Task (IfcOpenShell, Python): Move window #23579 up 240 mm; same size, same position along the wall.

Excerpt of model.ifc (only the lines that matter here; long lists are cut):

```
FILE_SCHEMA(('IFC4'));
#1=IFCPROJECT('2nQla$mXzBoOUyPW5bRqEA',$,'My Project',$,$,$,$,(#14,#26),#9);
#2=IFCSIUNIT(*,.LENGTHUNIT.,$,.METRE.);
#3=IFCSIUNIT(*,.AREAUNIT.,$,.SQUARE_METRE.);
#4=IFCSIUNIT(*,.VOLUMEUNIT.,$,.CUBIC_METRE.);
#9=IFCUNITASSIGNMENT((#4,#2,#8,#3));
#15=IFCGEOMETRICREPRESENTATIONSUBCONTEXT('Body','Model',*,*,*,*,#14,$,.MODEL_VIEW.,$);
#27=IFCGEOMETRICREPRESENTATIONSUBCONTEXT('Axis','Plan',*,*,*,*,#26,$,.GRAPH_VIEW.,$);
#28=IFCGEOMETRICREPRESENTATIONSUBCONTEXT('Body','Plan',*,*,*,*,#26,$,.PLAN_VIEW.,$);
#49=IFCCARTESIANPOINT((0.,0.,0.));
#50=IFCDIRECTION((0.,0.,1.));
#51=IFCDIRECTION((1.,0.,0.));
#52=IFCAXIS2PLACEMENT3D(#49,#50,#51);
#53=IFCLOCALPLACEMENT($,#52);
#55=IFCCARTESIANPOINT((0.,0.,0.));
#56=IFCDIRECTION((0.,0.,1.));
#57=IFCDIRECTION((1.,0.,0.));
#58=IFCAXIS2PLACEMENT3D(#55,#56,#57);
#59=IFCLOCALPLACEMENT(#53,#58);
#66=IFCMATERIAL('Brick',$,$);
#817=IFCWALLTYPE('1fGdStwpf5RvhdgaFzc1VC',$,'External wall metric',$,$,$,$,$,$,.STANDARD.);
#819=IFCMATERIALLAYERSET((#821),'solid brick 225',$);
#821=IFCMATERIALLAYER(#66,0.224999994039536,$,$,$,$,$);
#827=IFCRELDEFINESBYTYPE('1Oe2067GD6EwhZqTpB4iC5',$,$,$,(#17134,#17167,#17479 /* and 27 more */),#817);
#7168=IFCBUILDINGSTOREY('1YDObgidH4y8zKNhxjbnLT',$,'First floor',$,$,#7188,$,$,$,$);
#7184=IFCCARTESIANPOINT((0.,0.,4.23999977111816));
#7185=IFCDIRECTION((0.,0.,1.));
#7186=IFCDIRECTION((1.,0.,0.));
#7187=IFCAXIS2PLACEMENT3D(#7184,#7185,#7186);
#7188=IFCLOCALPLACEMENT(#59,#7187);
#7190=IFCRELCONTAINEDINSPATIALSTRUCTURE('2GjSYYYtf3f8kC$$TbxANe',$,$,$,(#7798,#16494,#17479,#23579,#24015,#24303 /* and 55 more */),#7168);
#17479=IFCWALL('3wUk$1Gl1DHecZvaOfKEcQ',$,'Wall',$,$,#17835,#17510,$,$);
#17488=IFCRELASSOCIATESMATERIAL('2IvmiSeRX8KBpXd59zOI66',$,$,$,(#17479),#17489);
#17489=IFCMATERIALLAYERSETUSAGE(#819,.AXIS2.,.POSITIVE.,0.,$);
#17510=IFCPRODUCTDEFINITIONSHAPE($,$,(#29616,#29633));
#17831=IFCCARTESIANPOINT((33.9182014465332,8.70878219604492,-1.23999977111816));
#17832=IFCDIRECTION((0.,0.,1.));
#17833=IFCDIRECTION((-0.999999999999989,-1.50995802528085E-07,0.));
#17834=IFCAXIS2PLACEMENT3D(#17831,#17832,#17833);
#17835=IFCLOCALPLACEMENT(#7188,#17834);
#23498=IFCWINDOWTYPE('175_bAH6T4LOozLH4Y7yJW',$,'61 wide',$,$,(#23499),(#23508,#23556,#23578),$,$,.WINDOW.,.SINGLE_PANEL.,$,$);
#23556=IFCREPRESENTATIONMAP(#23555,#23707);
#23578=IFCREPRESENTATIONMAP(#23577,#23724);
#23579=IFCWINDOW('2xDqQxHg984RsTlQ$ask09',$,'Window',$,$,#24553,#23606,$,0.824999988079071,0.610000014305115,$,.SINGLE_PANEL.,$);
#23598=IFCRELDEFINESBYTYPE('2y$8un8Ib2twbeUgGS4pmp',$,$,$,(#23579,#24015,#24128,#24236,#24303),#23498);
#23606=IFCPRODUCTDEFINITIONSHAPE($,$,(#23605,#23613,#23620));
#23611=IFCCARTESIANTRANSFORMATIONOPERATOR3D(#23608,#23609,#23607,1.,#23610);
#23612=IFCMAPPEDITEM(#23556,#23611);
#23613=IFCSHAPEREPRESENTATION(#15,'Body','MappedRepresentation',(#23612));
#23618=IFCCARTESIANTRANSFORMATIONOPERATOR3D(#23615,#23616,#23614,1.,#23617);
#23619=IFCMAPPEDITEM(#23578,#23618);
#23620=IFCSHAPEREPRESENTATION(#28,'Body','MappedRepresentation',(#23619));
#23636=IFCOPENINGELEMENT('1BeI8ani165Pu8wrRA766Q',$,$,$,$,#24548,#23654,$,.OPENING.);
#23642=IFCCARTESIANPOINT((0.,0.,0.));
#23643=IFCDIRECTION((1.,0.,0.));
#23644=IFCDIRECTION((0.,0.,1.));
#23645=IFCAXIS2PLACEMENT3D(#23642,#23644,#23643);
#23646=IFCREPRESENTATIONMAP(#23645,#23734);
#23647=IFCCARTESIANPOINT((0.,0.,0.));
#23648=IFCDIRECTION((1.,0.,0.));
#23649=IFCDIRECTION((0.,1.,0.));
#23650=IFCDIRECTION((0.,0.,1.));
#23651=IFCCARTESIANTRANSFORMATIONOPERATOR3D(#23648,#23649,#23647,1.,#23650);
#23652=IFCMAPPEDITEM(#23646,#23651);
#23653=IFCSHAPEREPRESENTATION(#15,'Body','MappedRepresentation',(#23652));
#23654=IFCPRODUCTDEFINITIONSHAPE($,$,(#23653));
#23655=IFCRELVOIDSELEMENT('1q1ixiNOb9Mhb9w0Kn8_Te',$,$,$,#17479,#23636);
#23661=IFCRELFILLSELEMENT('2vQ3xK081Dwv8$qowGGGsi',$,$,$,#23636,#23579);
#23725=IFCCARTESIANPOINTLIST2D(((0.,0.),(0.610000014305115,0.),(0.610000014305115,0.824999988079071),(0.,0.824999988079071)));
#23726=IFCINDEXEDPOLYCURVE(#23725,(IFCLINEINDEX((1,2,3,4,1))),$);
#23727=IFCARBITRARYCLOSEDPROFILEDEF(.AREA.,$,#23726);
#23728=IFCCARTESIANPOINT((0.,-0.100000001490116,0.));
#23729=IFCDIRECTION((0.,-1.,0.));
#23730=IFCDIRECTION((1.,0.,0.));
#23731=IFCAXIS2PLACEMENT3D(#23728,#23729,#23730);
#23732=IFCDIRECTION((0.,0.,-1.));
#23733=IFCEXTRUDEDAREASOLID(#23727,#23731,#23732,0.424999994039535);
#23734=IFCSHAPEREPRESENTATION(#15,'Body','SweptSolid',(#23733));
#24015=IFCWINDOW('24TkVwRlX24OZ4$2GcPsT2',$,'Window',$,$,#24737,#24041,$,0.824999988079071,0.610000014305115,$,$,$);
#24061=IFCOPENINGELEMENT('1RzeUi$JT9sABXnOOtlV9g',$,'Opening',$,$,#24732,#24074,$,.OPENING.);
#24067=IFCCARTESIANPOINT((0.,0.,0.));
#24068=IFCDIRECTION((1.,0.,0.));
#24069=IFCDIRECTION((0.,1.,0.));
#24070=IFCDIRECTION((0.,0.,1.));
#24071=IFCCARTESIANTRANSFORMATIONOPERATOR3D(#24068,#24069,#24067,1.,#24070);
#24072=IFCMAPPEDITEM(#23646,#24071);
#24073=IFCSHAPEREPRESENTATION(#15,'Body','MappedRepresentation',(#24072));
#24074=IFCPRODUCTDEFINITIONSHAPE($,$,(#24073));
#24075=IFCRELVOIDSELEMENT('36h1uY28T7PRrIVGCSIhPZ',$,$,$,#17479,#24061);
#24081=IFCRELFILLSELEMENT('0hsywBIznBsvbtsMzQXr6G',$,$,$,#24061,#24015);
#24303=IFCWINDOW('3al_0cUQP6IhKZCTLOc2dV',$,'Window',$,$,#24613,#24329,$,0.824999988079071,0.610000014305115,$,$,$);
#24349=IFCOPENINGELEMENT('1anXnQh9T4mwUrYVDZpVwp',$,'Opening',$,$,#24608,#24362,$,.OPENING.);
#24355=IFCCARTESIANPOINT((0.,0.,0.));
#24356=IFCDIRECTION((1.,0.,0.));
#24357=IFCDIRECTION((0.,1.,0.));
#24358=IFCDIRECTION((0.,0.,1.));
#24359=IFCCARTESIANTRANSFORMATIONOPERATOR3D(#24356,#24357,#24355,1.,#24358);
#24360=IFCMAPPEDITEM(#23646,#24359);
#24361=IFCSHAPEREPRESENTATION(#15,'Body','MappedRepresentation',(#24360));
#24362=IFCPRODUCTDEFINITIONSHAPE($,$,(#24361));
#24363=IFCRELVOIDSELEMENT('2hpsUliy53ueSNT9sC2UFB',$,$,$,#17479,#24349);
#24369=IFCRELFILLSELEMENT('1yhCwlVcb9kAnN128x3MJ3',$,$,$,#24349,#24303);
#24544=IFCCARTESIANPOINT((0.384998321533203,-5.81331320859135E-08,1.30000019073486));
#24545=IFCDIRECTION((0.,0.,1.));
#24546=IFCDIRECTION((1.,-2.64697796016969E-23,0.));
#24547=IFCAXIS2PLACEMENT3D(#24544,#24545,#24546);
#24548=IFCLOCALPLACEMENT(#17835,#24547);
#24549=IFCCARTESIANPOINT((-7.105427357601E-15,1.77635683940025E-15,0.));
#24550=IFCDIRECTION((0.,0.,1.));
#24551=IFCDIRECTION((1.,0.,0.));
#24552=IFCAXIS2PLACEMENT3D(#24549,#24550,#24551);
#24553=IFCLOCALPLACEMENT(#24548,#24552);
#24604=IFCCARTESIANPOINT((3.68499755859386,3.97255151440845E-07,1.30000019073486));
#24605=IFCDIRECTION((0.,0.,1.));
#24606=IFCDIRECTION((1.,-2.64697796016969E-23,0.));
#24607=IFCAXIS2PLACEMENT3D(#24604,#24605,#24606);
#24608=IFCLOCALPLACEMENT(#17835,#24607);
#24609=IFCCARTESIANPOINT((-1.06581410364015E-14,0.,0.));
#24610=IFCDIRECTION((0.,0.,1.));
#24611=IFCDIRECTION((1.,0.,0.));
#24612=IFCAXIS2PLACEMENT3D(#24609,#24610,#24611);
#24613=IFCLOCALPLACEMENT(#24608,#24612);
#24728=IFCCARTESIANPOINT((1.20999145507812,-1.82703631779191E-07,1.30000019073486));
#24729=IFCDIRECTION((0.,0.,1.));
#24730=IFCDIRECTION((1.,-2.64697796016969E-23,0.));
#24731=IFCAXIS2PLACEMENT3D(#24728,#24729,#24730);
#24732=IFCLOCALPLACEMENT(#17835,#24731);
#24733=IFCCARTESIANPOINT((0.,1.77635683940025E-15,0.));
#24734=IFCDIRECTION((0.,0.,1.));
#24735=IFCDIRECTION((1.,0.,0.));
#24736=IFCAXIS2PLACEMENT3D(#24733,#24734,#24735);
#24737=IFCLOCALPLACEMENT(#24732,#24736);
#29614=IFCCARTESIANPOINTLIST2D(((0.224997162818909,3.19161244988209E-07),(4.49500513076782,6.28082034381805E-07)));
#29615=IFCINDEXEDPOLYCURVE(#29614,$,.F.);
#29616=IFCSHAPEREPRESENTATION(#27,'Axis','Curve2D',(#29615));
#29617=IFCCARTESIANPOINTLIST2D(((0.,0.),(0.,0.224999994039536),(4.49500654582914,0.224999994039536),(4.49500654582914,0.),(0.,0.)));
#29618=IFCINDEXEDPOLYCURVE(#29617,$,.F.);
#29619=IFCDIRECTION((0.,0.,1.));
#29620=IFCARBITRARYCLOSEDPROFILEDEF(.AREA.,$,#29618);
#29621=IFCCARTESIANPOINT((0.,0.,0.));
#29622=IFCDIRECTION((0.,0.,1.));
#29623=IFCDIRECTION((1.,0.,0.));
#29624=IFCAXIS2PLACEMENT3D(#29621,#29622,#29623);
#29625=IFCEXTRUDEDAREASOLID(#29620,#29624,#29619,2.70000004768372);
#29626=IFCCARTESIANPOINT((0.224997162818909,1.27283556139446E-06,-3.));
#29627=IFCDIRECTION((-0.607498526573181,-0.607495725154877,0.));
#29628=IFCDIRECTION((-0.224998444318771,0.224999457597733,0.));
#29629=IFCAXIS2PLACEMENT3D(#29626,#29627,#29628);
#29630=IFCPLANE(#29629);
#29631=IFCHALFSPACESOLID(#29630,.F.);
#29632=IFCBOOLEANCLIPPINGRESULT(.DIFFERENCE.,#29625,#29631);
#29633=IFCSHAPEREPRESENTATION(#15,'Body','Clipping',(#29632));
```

```python
import numpy as np
import ifcopenshell
import ifcopenshell.api.geometry
import ifcopenshell.util.placement
import ifcopenshell.util.unit

model = ifcopenshell.open("model.ifc")
unit_scale = ifcopenshell.util.unit.calculate_unit_scale(model)

window = model.by_id(23579)
opening = window.FillsVoids[0].RelatingOpeningElement
dz = 0.24

shift = np.array([0.0, 0.0, dz])
# The window is placed relative to its opening, so it follows when the opening moves.
matrix = ifcopenshell.util.placement.get_local_placement(opening.ObjectPlacement)
matrix[:3, 3] += shift
ifcopenshell.api.geometry.edit_object_placement(
    model, product=opening, matrix=matrix, is_si=False, should_transform_children=True
)

print(f"moved by {dz * unit_scale:+.3f} m")

model.write("model_edited.ifc")
```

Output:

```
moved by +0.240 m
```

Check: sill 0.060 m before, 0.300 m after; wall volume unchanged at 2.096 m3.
